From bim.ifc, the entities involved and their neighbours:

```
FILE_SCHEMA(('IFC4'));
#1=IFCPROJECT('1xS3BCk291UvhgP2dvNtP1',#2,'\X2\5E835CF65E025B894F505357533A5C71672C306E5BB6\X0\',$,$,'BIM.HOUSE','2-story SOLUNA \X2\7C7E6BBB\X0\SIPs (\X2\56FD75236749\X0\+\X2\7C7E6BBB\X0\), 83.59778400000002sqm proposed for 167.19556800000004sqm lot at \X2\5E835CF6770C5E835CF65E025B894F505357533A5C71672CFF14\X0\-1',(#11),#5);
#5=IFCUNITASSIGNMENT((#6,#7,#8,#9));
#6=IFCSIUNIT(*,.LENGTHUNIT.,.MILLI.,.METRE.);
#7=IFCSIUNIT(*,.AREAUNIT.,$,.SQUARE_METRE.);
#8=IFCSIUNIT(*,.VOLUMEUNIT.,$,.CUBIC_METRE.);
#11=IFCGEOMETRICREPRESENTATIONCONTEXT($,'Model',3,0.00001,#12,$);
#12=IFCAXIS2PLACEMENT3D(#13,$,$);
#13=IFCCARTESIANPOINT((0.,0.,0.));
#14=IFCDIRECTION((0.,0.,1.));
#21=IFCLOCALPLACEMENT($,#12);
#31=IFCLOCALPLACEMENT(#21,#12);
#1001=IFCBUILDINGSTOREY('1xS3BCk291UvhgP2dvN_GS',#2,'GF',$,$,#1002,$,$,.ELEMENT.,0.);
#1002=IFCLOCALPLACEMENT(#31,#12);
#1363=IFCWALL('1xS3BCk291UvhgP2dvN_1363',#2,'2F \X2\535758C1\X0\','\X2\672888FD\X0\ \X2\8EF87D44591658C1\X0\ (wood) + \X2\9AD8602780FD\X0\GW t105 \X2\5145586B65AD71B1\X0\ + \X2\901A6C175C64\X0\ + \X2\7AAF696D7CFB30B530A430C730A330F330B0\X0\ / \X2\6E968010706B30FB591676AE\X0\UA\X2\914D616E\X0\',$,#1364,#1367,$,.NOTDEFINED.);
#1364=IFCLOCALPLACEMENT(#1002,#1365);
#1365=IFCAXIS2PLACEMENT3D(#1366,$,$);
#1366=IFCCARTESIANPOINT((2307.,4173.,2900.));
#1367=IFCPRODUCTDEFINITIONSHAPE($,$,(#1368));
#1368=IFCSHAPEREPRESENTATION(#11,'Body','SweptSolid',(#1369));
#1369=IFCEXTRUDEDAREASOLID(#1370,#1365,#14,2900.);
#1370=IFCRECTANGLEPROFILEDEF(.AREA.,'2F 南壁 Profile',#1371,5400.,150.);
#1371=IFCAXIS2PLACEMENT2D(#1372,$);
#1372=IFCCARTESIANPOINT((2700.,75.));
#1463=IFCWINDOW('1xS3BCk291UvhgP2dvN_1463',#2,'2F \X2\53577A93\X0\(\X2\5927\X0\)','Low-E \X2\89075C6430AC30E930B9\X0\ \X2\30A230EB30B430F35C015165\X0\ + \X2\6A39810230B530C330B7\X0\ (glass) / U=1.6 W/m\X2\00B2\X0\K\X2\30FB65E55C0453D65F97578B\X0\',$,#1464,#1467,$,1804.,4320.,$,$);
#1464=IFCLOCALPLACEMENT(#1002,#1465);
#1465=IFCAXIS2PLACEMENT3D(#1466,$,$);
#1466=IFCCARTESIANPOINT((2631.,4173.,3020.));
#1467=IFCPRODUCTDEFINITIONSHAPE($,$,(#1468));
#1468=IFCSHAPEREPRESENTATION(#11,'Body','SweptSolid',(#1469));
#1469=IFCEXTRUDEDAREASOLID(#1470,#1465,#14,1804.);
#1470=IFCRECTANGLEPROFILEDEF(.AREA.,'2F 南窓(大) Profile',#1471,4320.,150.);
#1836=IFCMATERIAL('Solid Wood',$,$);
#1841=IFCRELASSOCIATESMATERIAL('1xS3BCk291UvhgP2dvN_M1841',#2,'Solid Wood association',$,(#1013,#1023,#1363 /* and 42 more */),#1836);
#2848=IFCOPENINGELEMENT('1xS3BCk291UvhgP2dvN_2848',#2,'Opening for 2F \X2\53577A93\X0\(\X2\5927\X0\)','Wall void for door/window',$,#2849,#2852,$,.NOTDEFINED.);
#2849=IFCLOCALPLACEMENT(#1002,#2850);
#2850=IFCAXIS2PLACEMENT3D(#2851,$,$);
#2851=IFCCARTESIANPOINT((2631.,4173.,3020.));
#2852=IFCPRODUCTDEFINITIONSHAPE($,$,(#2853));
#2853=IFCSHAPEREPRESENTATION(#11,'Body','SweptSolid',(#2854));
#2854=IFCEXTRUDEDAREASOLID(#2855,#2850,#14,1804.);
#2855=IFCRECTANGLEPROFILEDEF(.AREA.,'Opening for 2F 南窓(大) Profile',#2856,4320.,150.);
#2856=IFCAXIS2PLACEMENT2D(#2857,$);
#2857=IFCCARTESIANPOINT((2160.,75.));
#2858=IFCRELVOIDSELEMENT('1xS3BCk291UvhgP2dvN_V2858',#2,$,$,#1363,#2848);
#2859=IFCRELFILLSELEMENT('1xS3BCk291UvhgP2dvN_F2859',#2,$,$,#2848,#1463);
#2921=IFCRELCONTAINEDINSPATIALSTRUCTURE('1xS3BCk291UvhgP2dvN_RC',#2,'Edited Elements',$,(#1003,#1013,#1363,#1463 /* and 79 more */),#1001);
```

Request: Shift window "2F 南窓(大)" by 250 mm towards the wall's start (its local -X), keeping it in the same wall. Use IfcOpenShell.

```python
import ifcopenshell
import ifcopenshell.api.geometry
import ifcopenshell.util.placement

model = ifcopenshell.open("bim.ifc")

window = model.by_guid("1xS3BCk291UvhgP2dvN_1463")
opening = window.FillsVoids[0].RelatingOpeningElement
wall = opening.VoidsElements[0].RelatingBuildingElement

wall_matrix = ifcopenshell.util.placement.get_local_placement(wall.ObjectPlacement)
shift = wall_matrix[:3, 0] * -250.0
before = ifcopenshell.util.placement.get_local_placement(window.ObjectPlacement)[:3, 3].copy()

# The window is not placed relative to its opening, so move both.
for product in (opening, window):
    matrix = ifcopenshell.util.placement.get_local_placement(product.ObjectPlacement)
    matrix[:3, 3] += shift
    ifcopenshell.api.geometry.edit_object_placement(model, product=product, matrix=matrix, is_si=False)

after = ifcopenshell.util.placement.get_local_placement(window.ObjectPlacement)[:3, 3]
print("window moved by", (after - before).round(3) + 0.0)

model.write("bim-out.ifc")
```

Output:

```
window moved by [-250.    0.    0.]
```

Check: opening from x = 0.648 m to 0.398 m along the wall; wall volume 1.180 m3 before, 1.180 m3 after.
